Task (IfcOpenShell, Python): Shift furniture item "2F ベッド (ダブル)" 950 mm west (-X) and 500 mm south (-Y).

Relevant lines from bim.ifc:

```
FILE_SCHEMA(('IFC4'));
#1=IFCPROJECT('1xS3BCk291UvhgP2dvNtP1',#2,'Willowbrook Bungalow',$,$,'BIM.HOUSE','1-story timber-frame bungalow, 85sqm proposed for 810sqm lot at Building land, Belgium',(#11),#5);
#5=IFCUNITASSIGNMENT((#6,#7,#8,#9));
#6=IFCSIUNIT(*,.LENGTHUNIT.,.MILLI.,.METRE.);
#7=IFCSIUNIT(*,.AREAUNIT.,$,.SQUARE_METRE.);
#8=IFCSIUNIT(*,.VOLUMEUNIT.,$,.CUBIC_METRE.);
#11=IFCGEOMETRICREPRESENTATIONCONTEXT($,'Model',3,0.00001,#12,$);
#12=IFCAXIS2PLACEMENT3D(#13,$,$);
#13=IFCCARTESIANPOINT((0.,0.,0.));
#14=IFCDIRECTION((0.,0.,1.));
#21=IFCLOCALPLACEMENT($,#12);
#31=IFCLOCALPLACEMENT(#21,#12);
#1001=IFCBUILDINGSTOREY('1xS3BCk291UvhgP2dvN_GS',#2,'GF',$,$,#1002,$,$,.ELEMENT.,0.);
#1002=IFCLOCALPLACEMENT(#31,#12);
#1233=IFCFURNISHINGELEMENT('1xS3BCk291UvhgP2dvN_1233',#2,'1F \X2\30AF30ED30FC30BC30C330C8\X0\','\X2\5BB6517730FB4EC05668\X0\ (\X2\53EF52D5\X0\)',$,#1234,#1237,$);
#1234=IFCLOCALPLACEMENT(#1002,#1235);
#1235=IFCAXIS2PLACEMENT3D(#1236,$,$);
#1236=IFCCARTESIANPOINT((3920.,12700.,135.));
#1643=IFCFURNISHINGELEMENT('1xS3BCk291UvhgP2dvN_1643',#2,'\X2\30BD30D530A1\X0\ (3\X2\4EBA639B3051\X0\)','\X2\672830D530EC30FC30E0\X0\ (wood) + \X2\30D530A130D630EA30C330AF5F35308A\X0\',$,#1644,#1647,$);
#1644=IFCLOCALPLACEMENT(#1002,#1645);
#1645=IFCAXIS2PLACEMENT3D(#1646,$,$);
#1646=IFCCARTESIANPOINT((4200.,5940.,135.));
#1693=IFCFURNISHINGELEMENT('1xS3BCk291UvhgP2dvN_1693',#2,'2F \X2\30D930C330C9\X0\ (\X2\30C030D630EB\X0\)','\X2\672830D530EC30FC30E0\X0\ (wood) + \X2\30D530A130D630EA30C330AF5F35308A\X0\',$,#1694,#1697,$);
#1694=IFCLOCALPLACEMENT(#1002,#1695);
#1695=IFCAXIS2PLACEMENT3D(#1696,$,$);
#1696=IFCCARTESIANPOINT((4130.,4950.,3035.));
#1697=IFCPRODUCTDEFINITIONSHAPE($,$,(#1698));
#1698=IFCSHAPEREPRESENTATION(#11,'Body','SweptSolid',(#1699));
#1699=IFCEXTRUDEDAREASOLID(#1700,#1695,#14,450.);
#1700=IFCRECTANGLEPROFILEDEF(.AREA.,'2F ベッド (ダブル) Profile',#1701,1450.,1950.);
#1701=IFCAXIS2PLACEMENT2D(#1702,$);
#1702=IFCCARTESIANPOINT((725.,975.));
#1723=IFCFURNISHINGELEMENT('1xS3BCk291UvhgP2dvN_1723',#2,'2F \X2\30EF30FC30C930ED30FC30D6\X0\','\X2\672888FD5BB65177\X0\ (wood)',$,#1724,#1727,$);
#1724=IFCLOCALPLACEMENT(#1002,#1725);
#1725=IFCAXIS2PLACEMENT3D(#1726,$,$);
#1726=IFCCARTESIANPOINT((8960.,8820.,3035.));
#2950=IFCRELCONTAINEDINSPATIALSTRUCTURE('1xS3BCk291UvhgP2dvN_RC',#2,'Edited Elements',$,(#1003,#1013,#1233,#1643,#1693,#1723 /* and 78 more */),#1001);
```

```python
import ifcopenshell
import ifcopenshell.api.geometry
import ifcopenshell.util.placement
import ifcopenshell.util.unit

model = ifcopenshell.open("bim.ifc")
unit_scale = ifcopenshell.util.unit.calculate_unit_scale(model)

item = model.by_id(1693)
matrix = ifcopenshell.util.placement.get_local_placement(item.ObjectPlacement)
matrix[0, 3] -= 0.95 / unit_scale
matrix[1, 3] -= 0.5 / unit_scale
ifcopenshell.api.geometry.edit_object_placement(model, product=item, matrix=matrix, is_si=False)

print(ifcopenshell.util.placement.get_local_placement(item.ObjectPlacement).round(3) + 0.0)

model.write("bim_v2.ifc")
```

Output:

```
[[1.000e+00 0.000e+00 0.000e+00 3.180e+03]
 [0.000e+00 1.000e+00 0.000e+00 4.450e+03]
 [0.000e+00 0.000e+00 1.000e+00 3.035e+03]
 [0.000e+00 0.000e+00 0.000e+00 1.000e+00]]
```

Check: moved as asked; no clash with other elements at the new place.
